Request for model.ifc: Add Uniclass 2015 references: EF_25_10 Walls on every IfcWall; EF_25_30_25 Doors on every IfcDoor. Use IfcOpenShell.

First a look at what the model holds.

```python
import ifcopenshell

model = ifcopenshell.open("model.ifc")
print(model.schema)
print("classifications:", [c.Name for c in model.by_type("IfcClassification")])
for ifc_class in ("IfcDoor", "IfcRoof", "IfcStair", "IfcWall", "IfcWindow"):
    print(ifc_class, len(model.by_type(ifc_class)))
```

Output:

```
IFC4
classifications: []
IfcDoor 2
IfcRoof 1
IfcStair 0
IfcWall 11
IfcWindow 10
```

```python
import ifcopenshell
import ifcopenshell.api.classification

model = ifcopenshell.open("model.ifc")

system = ifcopenshell.api.classification.add_classification(model, classification="Uniclass 2015")

codes = {
    "IfcWall": ("EF_25_10", "Walls"),
    "IfcDoor": ("EF_25_30_25", "Doors"),
}
for ifc_class, (code, name) in codes.items():
    products = model.by_type(ifc_class)
    ifcopenshell.api.classification.add_reference(
        model, products=products, classification=system, identification=code, name=name
    )
    print(code, len(products))

model.write("model_updated.ifc")
```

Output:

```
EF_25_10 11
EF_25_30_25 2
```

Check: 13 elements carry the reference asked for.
